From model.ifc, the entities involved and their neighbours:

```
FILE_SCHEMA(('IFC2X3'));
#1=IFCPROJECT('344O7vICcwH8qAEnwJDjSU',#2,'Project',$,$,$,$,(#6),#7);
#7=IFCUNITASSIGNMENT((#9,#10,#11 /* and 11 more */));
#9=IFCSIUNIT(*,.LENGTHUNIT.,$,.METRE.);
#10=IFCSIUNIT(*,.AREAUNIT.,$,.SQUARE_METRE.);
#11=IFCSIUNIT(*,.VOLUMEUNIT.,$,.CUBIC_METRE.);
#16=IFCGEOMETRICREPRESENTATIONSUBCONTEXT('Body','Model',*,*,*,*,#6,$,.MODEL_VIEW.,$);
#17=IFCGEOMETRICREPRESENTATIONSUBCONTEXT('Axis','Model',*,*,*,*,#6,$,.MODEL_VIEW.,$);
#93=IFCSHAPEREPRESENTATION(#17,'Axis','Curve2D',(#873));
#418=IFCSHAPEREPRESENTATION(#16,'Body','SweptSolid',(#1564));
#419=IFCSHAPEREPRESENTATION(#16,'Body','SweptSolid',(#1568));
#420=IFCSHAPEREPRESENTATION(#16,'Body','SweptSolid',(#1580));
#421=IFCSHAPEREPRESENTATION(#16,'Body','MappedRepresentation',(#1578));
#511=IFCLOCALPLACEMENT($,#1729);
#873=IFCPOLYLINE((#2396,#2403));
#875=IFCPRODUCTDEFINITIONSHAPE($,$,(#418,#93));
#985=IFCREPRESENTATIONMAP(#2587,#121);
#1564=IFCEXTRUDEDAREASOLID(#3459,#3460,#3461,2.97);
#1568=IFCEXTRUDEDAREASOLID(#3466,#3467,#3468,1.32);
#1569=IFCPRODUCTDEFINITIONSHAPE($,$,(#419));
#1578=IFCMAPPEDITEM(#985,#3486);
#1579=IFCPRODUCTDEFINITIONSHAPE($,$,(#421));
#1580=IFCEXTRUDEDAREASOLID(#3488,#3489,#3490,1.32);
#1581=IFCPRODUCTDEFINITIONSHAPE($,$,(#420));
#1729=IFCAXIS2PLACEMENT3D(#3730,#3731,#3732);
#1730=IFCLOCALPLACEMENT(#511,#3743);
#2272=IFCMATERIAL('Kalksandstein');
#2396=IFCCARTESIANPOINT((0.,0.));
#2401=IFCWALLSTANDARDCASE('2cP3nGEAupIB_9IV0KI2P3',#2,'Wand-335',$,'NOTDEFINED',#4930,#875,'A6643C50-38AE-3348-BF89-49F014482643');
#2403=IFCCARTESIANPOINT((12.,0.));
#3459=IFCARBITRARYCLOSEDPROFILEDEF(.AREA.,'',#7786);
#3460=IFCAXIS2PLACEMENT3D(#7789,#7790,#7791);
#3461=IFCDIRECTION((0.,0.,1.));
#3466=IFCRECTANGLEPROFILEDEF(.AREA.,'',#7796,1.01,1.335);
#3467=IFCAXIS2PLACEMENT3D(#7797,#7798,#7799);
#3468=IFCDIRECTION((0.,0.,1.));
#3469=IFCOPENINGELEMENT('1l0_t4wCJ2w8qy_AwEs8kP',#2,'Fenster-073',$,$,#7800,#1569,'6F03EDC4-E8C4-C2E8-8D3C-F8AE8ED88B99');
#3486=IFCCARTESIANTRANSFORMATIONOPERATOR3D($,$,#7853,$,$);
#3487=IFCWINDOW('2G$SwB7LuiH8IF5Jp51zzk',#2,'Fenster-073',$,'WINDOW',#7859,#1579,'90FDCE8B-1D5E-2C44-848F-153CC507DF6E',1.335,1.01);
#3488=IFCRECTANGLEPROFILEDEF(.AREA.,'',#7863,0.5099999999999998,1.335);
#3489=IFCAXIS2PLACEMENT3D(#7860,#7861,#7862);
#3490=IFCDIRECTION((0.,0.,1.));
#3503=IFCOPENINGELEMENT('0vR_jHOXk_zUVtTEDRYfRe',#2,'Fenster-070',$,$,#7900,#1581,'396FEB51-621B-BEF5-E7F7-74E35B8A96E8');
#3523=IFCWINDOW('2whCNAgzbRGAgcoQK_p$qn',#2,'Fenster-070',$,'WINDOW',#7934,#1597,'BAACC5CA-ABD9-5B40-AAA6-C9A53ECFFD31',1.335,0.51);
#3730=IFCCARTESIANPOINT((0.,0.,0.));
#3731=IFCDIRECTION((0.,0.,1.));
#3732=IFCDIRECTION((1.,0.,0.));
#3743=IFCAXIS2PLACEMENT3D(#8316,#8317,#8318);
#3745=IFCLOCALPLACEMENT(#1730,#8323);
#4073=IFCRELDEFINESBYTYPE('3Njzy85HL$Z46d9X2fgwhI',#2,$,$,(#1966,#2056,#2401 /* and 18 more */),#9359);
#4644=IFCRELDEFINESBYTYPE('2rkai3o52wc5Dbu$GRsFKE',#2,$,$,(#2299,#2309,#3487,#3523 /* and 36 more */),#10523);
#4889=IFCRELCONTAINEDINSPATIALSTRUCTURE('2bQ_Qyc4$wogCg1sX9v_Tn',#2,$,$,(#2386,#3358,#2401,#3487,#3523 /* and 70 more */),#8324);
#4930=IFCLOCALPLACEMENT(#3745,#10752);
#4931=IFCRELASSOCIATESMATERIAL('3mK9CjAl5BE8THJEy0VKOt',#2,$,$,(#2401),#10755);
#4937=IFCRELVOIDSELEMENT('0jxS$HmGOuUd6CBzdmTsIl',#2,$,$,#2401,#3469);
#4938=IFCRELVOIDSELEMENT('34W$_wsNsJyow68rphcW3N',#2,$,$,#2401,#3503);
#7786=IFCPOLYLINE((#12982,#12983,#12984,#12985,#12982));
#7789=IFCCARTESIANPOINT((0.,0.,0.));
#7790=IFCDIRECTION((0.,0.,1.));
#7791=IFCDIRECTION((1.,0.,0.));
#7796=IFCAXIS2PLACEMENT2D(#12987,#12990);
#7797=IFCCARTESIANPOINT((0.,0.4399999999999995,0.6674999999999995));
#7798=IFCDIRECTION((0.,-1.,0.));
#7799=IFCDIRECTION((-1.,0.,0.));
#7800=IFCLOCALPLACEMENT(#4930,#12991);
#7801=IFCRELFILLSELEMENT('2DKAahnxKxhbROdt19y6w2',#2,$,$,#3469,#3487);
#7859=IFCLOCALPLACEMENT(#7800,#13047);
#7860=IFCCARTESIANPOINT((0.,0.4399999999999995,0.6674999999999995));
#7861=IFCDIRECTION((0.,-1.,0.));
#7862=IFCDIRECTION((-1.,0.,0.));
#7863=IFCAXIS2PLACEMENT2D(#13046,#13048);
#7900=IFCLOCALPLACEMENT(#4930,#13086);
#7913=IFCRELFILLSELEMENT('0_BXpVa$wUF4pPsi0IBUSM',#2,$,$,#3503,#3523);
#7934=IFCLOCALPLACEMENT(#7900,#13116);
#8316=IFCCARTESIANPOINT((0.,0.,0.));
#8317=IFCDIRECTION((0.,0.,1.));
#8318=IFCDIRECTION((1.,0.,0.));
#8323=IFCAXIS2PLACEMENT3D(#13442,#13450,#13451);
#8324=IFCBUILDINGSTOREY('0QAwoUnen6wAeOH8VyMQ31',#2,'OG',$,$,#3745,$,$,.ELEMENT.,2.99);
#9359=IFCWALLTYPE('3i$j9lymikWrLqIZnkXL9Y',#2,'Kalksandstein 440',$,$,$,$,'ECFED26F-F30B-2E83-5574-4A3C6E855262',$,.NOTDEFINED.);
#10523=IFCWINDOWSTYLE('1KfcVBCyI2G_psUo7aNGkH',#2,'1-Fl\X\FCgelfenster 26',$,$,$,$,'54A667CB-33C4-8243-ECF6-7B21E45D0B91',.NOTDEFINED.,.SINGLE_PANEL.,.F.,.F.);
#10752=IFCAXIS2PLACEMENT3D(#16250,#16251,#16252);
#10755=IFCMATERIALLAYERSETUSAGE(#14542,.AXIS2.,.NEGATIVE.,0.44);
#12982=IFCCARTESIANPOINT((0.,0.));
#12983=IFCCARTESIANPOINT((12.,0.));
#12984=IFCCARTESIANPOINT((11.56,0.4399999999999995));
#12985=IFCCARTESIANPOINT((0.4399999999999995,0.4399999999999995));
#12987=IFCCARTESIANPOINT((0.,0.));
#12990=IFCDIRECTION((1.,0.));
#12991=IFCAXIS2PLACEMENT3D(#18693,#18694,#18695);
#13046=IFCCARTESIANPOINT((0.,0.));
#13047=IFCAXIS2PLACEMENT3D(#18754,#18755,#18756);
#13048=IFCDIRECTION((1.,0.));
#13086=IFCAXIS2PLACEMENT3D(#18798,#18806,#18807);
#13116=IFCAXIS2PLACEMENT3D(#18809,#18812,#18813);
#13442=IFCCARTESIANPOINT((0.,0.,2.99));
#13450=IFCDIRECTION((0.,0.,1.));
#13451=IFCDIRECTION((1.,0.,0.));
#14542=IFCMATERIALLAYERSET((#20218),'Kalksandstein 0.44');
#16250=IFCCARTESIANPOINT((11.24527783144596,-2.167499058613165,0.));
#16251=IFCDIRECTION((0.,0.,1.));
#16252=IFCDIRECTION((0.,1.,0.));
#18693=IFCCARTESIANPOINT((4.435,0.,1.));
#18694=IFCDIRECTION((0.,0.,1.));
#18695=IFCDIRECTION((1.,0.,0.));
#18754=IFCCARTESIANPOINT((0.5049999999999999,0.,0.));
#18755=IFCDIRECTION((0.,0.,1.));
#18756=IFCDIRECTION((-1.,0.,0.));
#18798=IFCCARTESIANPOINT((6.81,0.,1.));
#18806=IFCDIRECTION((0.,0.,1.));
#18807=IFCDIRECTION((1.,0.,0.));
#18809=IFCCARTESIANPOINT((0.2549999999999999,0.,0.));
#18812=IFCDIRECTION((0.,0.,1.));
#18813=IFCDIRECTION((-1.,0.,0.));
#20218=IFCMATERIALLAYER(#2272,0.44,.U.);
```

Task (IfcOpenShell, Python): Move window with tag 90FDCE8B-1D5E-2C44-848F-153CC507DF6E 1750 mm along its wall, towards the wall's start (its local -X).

```python
import ifcopenshell
import ifcopenshell.api.geometry
import ifcopenshell.util.placement
import ifcopenshell.util.unit

model = ifcopenshell.open("model.ifc")
unit_scale = ifcopenshell.util.unit.calculate_unit_scale(model)

window = model.by_id(3487)
opening = window.FillsVoids[0].RelatingOpeningElement
wall = opening.VoidsElements[0].RelatingBuildingElement

wall_matrix = ifcopenshell.util.placement.get_local_placement(wall.ObjectPlacement)
shift = wall_matrix[:3, 0] * -1.75 / unit_scale
before = ifcopenshell.util.placement.get_local_placement(window.ObjectPlacement)[:3, 3].copy()

# The window is placed relative to its opening, so it follows when the opening moves.
matrix = ifcopenshell.util.placement.get_local_placement(opening.ObjectPlacement)
matrix[:3, 3] += shift
ifcopenshell.api.geometry.edit_object_placement(
    model, product=opening, matrix=matrix, is_si=False, should_transform_children=True
)

after = ifcopenshell.util.placement.get_local_placement(window.ObjectPlacement)[:3, 3]
print("window moved by", (after - before).round(3) + 0.0)

model.write("model_rev.ifc")
```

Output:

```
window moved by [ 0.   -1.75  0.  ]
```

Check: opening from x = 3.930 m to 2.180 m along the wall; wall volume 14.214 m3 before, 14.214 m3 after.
